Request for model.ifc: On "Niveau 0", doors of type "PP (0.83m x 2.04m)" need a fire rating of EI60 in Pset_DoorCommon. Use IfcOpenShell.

First a look at what the model holds.

```python
import ifcopenshell
import ifcopenshell.util.element

model = ifcopenshell.open("model.ifc")
print(model.schema)
storey = next(s for s in model.by_type("IfcBuildingStorey") if s.Name == "Niveau 0")
doors = [e for e in ifcopenshell.util.element.get_decomposition(storey) if e.is_a("IfcDoor")]
seen = {}
for e in doors:
    element_type = ifcopenshell.util.element.get_type(e)
    key = (element_type.Name if element_type != e and element_type else None, ifcopenshell.util.element.get_pset(e, "Pset_DoorCommon", "FireRating"))
    seen[key] = seen.get(key, 0) + 1
for (name, value), count in sorted(seen.items(), key=str):
    print(count, "x", name, "|", value)
```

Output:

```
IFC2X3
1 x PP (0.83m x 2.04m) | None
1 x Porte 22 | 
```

```python
import ifcopenshell
import ifcopenshell.api.pset
import ifcopenshell.util.element

model = ifcopenshell.open("model.ifc")

storey = next(s for s in model.by_type("IfcBuildingStorey") if s.Name == "Niveau 0")
doors = [e for e in ifcopenshell.util.element.get_decomposition(storey) if e.is_a("IfcDoor")]

count = 0
for e in doors:
    element_type = ifcopenshell.util.element.get_type(e)
    if element_type in (None, e) or element_type.Name != "PP (0.83m x 2.04m)":
        continue
    # add_pset returns the element's existing set when there is one.
    pset = ifcopenshell.api.pset.add_pset(model, product=e, name="Pset_DoorCommon")
    ifcopenshell.api.pset.edit_pset(model, pset=pset, properties={"FireRating": "EI60"})
    count += 1

print(count, "doors updated")

model.write("model_edited.ifc")
```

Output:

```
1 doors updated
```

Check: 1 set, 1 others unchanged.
